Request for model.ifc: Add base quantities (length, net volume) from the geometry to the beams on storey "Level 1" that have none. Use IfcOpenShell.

First a look at what the model holds.

```python
import ifcopenshell
import ifcopenshell.util.element
import ifcopenshell.util.unit

model = ifcopenshell.open("model.ifc")
print(model.schema)
for unit_type in ("LENGTHUNIT", "AREAUNIT", "VOLUMEUNIT"):
    print(unit_type, ifcopenshell.util.unit.calculate_unit_scale(model, unit_type))
storey = next(s for s in model.by_type("IfcBuildingStorey") if s.Name == "Level 1")
beams = [e for e in ifcopenshell.util.element.get_decomposition(storey) if e.is_a("IfcBeam")]
for e in sorted(beams, key=lambda e: e.id()):
    print(e.id(), e.is_a(), e.Name, list(ifcopenshell.util.element.get_psets(e, qtos_only=True)), sep=" | ")
```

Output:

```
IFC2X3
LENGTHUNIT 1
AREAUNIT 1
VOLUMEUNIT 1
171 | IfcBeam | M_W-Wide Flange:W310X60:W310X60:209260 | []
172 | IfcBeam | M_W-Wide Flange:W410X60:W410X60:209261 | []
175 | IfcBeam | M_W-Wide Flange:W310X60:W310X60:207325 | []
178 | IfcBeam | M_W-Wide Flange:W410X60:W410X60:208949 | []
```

```python
import ifcopenshell
import ifcopenshell.api.pset
import ifcopenshell.geom
import ifcopenshell.util.element
import ifcopenshell.util.shape
import ifcopenshell.util.unit

model = ifcopenshell.open("model.ifc")
unit_scale = ifcopenshell.util.unit.calculate_unit_scale(model)
volume_scale = ifcopenshell.util.unit.calculate_unit_scale(model, "VOLUMEUNIT")
settings = ifcopenshell.geom.settings()

storey = next(s for s in model.by_type("IfcBuildingStorey") if s.Name == "Level 1")
beams = [e for e in ifcopenshell.util.element.get_decomposition(storey) if e.is_a("IfcBeam")]

for e in sorted(beams, key=lambda e: e.id()):
    if ifcopenshell.util.element.get_psets(e, qtos_only=True, should_inherit=False):
        continue
    # Geometry comes back in metres, in the element's own axes.
    shape = ifcopenshell.geom.create_shape(settings, e)
    values = {
        "Length": ifcopenshell.util.shape.get_max_xyz(shape.geometry) / unit_scale,
        "NetVolume": ifcopenshell.util.shape.get_volume(shape.geometry) / volume_scale,
    }
    qto = ifcopenshell.api.pset.add_qto(model, product=e, name="BaseQuantities")
    ifcopenshell.api.pset.edit_qto(model, qto=qto, properties=values)
    print(e.id(), {k: round(v, 3) for k, v in values.items()})

model.write("model_rev.ifc")
```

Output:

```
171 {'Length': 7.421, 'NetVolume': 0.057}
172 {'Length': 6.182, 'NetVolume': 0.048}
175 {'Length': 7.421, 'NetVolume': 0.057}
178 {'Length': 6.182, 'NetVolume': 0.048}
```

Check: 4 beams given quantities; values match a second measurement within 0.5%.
